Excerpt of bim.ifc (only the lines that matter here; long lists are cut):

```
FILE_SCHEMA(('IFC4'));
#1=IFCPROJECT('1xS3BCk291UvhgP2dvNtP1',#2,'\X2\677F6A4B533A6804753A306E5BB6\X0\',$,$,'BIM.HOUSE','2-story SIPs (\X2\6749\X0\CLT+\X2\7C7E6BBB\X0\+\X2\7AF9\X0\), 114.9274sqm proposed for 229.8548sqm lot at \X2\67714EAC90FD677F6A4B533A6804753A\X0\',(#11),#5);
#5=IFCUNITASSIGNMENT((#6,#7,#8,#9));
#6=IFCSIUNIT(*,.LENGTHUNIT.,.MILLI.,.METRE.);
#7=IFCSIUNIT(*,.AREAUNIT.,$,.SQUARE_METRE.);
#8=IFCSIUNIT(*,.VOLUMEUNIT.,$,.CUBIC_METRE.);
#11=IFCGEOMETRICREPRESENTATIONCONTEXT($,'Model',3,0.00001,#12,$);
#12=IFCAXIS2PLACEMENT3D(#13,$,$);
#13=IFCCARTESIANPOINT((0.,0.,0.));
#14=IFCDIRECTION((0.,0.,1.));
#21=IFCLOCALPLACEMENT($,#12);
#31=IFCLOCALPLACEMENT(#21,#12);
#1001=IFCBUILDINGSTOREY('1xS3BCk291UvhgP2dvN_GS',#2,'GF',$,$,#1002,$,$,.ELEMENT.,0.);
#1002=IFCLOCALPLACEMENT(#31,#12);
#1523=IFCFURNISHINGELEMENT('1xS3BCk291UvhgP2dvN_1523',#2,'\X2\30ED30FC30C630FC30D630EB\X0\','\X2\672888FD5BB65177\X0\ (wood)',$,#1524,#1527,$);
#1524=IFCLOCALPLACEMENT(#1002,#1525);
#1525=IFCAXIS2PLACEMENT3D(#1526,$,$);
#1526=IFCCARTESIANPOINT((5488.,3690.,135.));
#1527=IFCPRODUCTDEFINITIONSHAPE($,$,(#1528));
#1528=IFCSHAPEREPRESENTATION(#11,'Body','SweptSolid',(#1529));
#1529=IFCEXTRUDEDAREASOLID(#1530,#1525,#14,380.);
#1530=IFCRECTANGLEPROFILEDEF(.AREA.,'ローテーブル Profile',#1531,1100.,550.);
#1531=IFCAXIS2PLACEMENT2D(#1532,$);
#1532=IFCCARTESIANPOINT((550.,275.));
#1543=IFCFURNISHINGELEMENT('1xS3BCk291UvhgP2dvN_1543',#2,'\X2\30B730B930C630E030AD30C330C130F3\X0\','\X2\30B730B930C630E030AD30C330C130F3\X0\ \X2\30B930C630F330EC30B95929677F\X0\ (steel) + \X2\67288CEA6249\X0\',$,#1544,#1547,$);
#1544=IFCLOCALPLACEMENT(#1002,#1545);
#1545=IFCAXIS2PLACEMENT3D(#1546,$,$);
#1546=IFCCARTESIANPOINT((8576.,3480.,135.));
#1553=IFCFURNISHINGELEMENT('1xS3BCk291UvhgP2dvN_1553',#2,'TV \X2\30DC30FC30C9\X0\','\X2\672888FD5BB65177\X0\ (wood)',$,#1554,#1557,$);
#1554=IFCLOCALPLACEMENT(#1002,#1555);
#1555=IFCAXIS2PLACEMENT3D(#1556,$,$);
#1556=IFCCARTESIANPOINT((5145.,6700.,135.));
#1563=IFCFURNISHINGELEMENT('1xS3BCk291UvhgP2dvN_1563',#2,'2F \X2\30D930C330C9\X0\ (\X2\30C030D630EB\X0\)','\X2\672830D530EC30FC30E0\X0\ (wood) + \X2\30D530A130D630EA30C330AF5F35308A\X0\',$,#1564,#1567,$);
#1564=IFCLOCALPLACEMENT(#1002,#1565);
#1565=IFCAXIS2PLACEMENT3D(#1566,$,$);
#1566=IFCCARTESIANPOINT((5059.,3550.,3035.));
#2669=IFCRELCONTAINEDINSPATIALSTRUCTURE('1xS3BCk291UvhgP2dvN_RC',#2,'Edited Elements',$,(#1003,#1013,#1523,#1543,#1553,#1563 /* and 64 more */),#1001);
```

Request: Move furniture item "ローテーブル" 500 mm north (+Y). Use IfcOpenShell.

```python
import ifcopenshell
import ifcopenshell.api.geometry
import ifcopenshell.util.placement

model = ifcopenshell.open("bim.ifc")

item = model.by_guid("1xS3BCk291UvhgP2dvN_1523")
matrix = ifcopenshell.util.placement.get_local_placement(item.ObjectPlacement)
matrix[1, 3] += 500.0
ifcopenshell.api.geometry.edit_object_placement(model, product=item, matrix=matrix, is_si=False)

print(ifcopenshell.util.placement.get_local_placement(item.ObjectPlacement).round(3) + 0.0)

model.write("bim-out.ifc")
```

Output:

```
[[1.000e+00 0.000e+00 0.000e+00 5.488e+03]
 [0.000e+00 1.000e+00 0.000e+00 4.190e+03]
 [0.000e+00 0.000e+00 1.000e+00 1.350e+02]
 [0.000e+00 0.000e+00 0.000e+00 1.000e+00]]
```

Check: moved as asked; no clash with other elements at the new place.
